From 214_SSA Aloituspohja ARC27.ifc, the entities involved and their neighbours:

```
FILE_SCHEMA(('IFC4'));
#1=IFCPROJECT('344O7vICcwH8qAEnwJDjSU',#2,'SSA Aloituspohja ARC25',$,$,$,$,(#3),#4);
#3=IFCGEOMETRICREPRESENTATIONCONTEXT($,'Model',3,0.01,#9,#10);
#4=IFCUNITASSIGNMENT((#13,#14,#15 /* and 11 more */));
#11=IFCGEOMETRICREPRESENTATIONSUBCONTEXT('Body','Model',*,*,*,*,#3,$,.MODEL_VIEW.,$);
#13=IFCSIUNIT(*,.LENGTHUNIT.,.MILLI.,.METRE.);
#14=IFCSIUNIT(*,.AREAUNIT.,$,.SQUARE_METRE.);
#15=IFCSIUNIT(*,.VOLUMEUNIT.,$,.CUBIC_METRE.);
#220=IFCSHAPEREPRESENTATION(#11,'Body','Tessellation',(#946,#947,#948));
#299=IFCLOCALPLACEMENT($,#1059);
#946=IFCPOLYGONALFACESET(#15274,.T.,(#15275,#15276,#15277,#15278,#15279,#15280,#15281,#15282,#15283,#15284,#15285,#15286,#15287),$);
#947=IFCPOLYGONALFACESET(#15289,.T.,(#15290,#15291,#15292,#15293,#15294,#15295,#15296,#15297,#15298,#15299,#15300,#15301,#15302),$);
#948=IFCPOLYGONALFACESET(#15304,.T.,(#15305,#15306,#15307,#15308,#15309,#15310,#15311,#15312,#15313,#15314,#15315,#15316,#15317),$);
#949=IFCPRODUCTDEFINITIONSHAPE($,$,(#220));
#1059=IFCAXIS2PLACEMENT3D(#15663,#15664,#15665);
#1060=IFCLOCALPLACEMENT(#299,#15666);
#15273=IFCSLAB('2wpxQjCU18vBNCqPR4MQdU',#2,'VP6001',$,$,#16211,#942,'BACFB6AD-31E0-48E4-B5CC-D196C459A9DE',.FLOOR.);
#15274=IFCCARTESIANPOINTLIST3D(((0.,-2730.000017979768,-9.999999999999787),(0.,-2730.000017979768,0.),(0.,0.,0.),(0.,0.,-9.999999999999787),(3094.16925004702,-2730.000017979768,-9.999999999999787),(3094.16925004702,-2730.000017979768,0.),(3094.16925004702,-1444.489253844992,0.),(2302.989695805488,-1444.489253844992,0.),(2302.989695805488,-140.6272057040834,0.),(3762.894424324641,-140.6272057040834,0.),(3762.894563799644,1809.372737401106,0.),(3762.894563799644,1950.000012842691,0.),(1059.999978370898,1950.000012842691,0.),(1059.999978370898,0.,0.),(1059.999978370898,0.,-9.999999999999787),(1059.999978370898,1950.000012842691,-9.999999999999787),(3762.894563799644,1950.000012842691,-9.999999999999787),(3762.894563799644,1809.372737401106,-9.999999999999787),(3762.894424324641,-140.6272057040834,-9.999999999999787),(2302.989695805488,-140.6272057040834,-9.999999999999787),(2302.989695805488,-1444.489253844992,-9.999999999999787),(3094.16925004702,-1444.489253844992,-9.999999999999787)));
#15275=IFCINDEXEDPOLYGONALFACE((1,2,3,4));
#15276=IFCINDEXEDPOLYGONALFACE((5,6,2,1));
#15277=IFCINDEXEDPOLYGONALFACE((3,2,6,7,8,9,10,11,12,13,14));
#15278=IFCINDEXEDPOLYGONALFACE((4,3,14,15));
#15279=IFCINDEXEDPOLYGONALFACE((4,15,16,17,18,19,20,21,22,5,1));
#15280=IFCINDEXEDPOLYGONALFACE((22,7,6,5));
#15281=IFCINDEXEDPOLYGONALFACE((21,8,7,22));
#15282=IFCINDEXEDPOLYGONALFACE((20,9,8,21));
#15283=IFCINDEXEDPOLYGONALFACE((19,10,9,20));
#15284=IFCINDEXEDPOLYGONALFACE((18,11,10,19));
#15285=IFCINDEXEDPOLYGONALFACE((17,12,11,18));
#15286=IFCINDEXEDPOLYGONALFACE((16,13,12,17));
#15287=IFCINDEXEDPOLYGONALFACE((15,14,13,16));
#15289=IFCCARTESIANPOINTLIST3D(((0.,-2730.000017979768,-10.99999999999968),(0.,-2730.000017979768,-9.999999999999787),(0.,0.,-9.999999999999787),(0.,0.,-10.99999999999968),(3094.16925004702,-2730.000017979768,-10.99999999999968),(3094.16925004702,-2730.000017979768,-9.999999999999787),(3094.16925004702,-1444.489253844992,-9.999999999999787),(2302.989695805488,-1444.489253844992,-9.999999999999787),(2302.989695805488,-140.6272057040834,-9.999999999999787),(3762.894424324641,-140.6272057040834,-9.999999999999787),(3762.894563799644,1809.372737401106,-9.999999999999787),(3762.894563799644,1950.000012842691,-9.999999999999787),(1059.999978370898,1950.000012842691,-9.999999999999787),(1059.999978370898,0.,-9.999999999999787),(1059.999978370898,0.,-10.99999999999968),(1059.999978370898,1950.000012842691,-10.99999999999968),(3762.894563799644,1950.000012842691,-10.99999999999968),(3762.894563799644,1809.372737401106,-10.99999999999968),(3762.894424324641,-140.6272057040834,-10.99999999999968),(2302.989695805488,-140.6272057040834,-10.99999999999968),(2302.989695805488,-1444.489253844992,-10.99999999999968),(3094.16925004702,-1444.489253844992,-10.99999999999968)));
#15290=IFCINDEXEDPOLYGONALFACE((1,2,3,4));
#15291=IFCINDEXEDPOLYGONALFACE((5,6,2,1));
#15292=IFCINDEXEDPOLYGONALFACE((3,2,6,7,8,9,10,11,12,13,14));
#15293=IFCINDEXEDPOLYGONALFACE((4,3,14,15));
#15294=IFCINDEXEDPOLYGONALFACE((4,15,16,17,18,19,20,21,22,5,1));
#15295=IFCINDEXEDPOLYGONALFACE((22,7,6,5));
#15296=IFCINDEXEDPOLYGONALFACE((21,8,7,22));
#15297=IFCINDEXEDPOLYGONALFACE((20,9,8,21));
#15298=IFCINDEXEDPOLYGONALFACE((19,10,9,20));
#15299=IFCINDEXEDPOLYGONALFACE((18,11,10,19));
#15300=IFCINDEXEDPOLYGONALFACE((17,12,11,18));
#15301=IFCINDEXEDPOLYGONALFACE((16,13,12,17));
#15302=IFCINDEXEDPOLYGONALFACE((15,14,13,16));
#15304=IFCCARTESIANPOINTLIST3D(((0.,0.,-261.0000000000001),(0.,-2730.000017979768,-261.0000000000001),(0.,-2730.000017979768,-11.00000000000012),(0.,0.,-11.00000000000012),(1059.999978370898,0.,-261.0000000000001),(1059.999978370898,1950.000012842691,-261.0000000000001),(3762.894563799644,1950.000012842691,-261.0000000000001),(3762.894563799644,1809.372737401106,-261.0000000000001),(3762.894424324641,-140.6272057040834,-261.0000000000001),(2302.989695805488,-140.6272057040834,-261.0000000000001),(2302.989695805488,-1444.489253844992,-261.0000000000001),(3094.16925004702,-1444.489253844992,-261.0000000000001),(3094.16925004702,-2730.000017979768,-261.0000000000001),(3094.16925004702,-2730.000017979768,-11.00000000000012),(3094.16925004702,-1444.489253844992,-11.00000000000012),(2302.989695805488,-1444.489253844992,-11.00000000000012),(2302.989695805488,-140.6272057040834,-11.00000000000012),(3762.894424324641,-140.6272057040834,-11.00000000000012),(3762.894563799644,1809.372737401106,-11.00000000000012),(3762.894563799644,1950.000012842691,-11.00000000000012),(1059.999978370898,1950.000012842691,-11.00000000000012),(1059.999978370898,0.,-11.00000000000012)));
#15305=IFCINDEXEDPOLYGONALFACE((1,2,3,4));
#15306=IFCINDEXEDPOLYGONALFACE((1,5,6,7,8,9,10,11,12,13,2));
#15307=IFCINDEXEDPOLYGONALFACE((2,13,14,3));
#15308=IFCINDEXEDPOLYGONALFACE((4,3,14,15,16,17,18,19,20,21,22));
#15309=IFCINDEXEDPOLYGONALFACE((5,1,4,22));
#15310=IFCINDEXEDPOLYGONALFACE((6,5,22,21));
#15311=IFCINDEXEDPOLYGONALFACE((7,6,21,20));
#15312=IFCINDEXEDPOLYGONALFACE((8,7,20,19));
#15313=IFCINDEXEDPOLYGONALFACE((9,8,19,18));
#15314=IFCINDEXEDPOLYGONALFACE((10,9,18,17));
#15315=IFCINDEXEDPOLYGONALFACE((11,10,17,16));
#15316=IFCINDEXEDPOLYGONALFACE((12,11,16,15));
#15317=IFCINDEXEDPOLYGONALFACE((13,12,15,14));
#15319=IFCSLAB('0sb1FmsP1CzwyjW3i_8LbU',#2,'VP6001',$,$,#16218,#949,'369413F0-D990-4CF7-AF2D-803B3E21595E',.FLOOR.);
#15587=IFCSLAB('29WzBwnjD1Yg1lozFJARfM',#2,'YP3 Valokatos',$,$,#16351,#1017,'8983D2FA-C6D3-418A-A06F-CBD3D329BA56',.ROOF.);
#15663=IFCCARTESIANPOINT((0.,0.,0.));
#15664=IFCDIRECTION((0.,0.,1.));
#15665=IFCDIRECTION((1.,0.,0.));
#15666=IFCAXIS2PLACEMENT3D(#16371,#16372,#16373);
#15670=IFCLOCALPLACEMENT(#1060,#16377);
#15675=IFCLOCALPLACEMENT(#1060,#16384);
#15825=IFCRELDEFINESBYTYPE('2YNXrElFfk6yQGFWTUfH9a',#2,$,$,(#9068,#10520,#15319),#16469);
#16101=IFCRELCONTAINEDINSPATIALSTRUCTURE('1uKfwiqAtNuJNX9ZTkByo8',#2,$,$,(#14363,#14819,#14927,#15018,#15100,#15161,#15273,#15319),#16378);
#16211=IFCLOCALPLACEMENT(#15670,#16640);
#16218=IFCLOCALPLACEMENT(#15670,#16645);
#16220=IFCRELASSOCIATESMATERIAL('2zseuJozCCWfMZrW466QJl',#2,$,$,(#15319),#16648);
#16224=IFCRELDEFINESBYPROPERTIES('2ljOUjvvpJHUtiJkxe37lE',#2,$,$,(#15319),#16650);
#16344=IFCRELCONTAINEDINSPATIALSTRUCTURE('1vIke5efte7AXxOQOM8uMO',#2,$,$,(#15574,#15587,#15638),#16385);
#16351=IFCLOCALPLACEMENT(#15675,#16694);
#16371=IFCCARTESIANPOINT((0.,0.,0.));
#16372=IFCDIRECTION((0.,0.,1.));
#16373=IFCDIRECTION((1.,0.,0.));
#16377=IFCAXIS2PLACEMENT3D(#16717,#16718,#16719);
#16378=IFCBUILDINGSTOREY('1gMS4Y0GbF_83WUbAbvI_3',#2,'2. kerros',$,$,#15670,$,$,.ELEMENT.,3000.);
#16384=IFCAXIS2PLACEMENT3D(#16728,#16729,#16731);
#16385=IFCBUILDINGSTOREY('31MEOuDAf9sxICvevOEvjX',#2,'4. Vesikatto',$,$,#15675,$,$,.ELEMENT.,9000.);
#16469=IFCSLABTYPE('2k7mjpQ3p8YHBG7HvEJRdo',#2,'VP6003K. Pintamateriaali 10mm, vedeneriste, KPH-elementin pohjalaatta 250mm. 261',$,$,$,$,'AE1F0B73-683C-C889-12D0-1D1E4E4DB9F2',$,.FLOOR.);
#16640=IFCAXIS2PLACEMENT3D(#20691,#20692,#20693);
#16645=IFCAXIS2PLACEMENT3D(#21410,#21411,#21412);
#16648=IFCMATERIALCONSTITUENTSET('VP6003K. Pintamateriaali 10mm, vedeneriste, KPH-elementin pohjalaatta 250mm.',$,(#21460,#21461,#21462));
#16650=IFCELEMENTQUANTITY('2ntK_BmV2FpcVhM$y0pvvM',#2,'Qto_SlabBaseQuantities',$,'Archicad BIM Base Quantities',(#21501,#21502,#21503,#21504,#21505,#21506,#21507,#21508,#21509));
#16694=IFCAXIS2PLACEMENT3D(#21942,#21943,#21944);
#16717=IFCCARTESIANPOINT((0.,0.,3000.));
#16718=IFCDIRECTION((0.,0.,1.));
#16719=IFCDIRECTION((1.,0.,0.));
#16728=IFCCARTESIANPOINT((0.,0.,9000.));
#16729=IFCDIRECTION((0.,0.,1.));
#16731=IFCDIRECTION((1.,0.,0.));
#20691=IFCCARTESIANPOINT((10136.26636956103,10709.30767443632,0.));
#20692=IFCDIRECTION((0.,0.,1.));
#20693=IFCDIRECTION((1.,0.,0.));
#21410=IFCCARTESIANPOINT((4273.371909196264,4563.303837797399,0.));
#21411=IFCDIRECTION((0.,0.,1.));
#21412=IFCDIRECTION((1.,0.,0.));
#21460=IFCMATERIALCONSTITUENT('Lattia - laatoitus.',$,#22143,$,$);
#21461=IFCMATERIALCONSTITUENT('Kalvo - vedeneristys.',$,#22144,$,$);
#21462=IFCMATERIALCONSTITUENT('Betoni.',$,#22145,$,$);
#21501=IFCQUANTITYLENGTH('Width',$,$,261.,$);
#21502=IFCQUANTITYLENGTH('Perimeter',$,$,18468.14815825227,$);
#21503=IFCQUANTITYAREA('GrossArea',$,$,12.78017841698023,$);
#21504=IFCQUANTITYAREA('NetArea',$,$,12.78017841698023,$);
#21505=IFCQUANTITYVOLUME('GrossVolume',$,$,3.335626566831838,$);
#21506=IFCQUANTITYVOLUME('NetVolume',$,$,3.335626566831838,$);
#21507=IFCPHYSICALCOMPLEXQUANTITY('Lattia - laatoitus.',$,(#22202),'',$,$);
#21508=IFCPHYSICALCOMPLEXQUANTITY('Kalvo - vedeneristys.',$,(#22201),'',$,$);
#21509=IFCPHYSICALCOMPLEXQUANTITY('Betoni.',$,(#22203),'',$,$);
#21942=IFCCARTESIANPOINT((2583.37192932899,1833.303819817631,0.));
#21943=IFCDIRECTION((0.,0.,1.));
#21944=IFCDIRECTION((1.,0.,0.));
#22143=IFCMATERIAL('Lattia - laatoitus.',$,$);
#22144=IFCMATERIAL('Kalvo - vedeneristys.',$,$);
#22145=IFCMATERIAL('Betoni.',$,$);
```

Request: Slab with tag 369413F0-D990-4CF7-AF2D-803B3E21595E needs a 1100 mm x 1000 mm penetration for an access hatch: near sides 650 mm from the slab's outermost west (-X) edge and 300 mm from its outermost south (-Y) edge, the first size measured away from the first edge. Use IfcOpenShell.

```python
import numpy as np
import ifcopenshell
import ifcopenshell.api.feature
import ifcopenshell.api.geometry
import ifcopenshell.api.pset
import ifcopenshell.api.root
import ifcopenshell.geom
import ifcopenshell.util.element
import ifcopenshell.util.placement
import ifcopenshell.util.representation
import ifcopenshell.util.shape
import ifcopenshell.util.unit

model = ifcopenshell.open("214_SSA Aloituspohja ARC27.ifc")
unit_scale = ifcopenshell.util.unit.calculate_unit_scale(model)
area_scale = ifcopenshell.util.unit.calculate_unit_scale(model, "AREAUNIT")
volume_scale = ifcopenshell.util.unit.calculate_unit_scale(model, "VOLUMEUNIT")
settings = ifcopenshell.geom.settings()


def volume(element):
    """Net volume in cubic metres, openings subtracted."""
    shape = ifcopenshell.geom.create_shape(settings, element)
    return ifcopenshell.util.shape.get_volume(shape.geometry)


slab = model.by_id(15319)
before = volume(slab)

# Extent in the slab's own axes, in metres. The edges named are its -X and -Y sides.
slab_shape = ifcopenshell.geom.create_shape(settings, slab)
vertices = ifcopenshell.util.shape.get_vertices(slab_shape.geometry)
x_min, y_min, bottom = vertices.min(axis=0)
top = vertices[:, 2].max()

opening = ifcopenshell.api.root.create_entity(model, ifc_class="IfcOpeningElement", name="Access hatch opening", predefined_type="OPENING")
context = ifcopenshell.util.representation.get_context(model, "Model", "Body", "MODEL_VIEW")
width, depth = 1.1, 1
outline = [(0.0, 0.0), (width, 0.0), (width, depth), (0.0, depth), (0.0, 0.0)]
# Overshoot both faces by 50 mm so the cut is clean.
shape = ifcopenshell.api.geometry.add_slab_representation(
    model, context=context, depth=top - bottom + 0.1, polyline=outline
)
ifcopenshell.api.geometry.assign_representation(model, product=opening, representation=shape)

matrix = ifcopenshell.util.placement.get_local_placement(slab.ObjectPlacement)
matrix[:, 3] = matrix @ np.append(np.array([x_min + 0.65, y_min + 0.3, bottom - 0.05]) / unit_scale, 1.0)
ifcopenshell.api.geometry.edit_object_placement(model, product=opening, matrix=matrix, is_si=False)
ifcopenshell.api.feature.add_feature(model, feature=opening, element=slab)

after = volume(slab)

# Update the slab's stored quantities.
qto = model.by_id(ifcopenshell.util.element.get_pset(slab, "Qto_SlabBaseQuantities", should_inherit=False)["id"])
ifcopenshell.api.pset.edit_qto(model, qto=qto, properties={
    "NetArea": after / (top - bottom) / area_scale,
    "NetVolume": after / volume_scale,
})

print(f"slab volume {before:.3f} -> {after:.3f} m3")

model.write("214_SSA Aloituspohja ARC27_updated.ifc")
```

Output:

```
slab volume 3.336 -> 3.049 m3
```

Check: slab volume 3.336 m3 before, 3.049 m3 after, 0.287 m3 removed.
